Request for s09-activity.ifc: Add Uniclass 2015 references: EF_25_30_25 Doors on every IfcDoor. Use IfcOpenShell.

First a look at what the model holds.

```python
import ifcopenshell

model = ifcopenshell.open("s09-activity.ifc")
print(model.schema)
print("classifications:", [c.Name for c in model.by_type("IfcClassification")])
for ifc_class in ("IfcDoor", "IfcRoof", "IfcStair", "IfcWall", "IfcWindow"):
    print(ifc_class, len(model.by_type(ifc_class)))
```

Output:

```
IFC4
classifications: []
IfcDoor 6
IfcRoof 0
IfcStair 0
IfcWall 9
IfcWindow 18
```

```python
import ifcopenshell
import ifcopenshell.api.classification

model = ifcopenshell.open("s09-activity.ifc")

system = ifcopenshell.api.classification.add_classification(model, classification="Uniclass 2015")

codes = {
    "IfcDoor": ("EF_25_30_25", "Doors"),
}
for ifc_class, (code, name) in codes.items():
    products = model.by_type(ifc_class)
    ifcopenshell.api.classification.add_reference(
        model, products=products, classification=system, identification=code, name=name
    )
    print(code, len(products))

model.write("s09-activity_v2.ifc")
```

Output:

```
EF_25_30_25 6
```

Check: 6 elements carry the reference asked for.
